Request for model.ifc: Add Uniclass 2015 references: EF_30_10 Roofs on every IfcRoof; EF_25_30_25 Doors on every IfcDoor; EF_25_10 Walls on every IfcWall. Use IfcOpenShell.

First a look at what the model holds.

```python
import ifcopenshell

model = ifcopenshell.open("model.ifc")
print(model.schema)
print("classifications:", [c.Name for c in model.by_type("IfcClassification")])
for ifc_class in ("IfcDoor", "IfcRoof", "IfcStair", "IfcWall", "IfcWindow"):
    print(ifc_class, len(model.by_type(ifc_class)))
```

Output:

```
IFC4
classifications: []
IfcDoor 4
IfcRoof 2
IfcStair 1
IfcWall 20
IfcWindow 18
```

```python
import ifcopenshell
import ifcopenshell.api.classification

model = ifcopenshell.open("model.ifc")

system = ifcopenshell.api.classification.add_classification(model, classification="Uniclass 2015")

codes = {
    "IfcRoof": ("EF_30_10", "Roofs"),
    "IfcDoor": ("EF_25_30_25", "Doors"),
    "IfcWall": ("EF_25_10", "Walls"),
}
for ifc_class, (code, name) in codes.items():
    products = model.by_type(ifc_class)
    ifcopenshell.api.classification.add_reference(
        model, products=products, classification=system, identification=code, name=name
    )
    print(code, len(products))

model.write("model-out.ifc")
```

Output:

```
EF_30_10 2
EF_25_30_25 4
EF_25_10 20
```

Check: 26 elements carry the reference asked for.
